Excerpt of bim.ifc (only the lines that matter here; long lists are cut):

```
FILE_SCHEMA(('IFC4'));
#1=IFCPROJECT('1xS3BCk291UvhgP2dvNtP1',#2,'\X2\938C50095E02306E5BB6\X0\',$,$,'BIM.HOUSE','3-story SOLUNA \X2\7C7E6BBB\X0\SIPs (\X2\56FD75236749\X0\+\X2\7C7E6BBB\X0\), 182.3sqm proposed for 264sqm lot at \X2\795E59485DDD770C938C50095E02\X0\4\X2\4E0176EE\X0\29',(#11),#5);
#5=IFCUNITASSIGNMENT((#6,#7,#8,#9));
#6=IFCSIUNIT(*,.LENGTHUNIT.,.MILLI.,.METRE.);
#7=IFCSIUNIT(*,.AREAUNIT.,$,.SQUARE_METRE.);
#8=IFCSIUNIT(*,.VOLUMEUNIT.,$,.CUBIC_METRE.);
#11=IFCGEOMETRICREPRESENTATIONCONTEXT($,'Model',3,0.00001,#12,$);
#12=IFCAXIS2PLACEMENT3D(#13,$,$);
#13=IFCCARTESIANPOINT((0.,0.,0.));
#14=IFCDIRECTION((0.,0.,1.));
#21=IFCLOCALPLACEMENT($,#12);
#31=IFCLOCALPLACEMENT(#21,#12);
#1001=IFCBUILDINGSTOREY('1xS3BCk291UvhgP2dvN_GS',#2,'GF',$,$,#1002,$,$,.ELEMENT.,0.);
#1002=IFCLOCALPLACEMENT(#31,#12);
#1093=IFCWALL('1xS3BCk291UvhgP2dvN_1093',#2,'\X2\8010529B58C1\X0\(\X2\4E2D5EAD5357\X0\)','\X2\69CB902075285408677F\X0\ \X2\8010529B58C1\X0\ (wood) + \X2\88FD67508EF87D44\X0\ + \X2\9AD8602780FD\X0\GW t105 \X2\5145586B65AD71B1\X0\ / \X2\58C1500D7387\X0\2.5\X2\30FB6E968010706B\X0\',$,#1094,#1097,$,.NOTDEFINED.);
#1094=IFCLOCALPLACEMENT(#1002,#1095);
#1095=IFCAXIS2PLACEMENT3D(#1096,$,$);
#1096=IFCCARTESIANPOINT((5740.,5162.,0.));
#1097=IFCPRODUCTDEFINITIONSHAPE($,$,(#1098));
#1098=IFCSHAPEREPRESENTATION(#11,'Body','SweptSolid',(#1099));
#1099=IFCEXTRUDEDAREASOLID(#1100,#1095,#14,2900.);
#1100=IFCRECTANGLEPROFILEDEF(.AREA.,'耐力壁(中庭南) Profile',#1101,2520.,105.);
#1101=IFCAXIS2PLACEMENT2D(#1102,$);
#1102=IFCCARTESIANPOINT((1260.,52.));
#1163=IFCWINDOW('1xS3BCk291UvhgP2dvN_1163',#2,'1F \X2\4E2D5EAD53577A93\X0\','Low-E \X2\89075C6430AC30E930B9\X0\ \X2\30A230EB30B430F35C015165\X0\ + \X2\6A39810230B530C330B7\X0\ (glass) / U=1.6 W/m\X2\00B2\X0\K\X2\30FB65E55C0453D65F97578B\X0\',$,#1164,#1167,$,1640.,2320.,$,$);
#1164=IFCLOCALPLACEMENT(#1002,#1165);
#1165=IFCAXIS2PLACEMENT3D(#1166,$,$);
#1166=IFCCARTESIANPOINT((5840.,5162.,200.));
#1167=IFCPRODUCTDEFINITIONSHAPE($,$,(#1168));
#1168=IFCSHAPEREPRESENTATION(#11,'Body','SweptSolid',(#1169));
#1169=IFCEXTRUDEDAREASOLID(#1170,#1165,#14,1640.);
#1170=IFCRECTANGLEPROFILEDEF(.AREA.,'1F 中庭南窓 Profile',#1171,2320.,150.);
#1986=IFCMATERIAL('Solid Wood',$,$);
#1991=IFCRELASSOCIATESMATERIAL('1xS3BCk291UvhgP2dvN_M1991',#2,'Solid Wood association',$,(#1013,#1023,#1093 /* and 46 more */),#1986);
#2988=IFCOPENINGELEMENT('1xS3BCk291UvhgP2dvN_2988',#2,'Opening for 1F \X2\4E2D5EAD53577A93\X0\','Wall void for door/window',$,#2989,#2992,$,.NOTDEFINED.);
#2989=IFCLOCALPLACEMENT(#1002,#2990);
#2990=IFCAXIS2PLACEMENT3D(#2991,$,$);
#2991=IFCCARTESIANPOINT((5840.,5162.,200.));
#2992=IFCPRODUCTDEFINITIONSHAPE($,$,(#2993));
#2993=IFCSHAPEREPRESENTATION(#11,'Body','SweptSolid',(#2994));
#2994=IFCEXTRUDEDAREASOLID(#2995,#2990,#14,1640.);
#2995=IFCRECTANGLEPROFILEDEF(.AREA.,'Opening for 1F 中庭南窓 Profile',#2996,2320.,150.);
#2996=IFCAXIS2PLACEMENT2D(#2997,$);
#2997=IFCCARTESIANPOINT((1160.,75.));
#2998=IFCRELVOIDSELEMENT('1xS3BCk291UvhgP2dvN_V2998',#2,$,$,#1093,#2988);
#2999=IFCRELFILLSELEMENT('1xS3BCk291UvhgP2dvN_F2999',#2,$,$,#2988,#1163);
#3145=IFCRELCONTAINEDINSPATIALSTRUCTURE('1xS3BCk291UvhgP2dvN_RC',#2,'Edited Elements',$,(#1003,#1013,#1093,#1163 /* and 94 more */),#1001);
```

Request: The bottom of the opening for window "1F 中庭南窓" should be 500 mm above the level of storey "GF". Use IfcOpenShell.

```python
import numpy as np
import ifcopenshell
import ifcopenshell.api.geometry
import ifcopenshell.geom
import ifcopenshell.util.element
import ifcopenshell.util.placement
import ifcopenshell.util.shape
import ifcopenshell.util.unit

model = ifcopenshell.open("bim.ifc")
unit_scale = ifcopenshell.util.unit.calculate_unit_scale(model)

window = model.by_guid("1xS3BCk291UvhgP2dvN_1163")
opening = window.FillsVoids[0].RelatingOpeningElement
storey = ifcopenshell.util.element.get_container(window, ifc_class="IfcBuildingStorey")
level = ifcopenshell.util.placement.get_local_placement(storey.ObjectPlacement)[2, 3]

# The opening's origin need not be at the sill, so measure its lowest point.
shape = ifcopenshell.geom.create_shape(ifcopenshell.geom.settings(), opening)
bottom = ifcopenshell.util.shape.get_shape_bottom_elevation(shape, shape.geometry) / unit_scale
dz = level + 0.5 / unit_scale - bottom

shift = np.array([0.0, 0.0, dz])
# The window is not placed relative to its opening, so move both.
for product in (opening, window):
    matrix = ifcopenshell.util.placement.get_local_placement(product.ObjectPlacement)
    matrix[:3, 3] += shift
    ifcopenshell.api.geometry.edit_object_placement(model, product=product, matrix=matrix, is_si=False)

print(f"moved by {dz * unit_scale:+.3f} m")

model.write("bim-out.ifc")
```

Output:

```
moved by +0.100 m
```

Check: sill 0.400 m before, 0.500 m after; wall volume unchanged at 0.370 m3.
